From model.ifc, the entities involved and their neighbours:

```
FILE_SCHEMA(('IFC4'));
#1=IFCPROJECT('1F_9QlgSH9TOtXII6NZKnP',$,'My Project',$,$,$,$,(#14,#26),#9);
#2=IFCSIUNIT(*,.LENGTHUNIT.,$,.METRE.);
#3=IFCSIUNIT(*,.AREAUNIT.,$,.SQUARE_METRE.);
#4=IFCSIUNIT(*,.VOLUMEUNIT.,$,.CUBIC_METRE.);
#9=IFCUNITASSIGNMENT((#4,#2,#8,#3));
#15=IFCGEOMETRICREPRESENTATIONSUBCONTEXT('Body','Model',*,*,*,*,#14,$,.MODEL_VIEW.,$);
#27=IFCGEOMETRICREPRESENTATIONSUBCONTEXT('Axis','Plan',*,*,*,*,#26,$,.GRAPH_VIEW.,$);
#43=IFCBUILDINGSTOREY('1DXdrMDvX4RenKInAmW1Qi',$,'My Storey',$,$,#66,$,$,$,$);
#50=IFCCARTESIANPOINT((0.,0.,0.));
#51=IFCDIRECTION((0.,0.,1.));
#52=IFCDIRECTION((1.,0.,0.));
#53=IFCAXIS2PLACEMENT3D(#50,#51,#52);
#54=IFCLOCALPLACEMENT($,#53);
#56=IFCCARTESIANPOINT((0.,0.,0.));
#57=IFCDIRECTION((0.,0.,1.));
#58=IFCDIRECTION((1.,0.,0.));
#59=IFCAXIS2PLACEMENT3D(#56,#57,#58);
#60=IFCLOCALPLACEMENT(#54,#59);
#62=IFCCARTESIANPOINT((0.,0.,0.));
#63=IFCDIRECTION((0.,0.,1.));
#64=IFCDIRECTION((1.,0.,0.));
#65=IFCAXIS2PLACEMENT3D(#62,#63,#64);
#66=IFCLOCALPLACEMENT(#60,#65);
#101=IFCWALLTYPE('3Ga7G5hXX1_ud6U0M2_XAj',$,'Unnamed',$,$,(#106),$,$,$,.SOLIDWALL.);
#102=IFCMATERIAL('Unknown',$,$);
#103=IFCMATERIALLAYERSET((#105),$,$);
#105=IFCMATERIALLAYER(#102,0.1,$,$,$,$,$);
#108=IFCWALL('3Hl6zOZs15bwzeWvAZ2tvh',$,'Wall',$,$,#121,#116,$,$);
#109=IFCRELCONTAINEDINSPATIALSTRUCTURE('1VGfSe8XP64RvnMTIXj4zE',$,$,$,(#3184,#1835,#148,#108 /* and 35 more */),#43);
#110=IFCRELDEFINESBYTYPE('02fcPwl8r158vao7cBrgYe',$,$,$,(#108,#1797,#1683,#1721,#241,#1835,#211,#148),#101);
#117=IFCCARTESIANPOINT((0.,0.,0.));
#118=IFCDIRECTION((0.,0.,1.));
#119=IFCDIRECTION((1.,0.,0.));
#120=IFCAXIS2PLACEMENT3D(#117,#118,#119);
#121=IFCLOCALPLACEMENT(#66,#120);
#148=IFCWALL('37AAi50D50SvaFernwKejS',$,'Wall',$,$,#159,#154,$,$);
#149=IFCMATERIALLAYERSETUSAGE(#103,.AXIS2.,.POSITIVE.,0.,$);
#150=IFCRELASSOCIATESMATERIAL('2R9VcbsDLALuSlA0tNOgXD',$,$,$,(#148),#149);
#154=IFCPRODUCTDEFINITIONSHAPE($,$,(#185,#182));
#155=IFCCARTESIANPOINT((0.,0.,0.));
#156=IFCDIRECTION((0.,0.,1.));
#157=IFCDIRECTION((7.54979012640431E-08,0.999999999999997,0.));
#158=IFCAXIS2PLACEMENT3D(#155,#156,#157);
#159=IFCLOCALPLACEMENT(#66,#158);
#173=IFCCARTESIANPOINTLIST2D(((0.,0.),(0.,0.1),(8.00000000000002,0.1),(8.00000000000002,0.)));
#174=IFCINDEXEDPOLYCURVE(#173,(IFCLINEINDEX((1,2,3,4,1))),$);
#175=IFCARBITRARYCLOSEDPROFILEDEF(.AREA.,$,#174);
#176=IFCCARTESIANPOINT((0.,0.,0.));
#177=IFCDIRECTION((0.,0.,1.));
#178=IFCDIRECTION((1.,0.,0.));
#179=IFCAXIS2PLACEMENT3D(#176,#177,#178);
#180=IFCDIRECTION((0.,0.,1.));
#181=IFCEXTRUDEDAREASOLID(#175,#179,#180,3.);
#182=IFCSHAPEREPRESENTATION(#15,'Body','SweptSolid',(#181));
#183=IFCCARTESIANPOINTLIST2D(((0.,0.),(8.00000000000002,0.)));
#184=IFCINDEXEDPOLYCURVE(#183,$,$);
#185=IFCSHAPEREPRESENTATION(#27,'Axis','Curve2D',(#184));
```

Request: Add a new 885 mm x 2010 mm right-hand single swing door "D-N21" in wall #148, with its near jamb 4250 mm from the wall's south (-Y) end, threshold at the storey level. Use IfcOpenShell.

```python
import numpy as np
import ifcopenshell
import ifcopenshell.api.feature
import ifcopenshell.api.geometry
import ifcopenshell.api.root
import ifcopenshell.api.spatial
import ifcopenshell.geom
import ifcopenshell.util.element
import ifcopenshell.util.placement
import ifcopenshell.util.representation
import ifcopenshell.util.shape
import ifcopenshell.util.unit

model = ifcopenshell.open("model.ifc")
unit_scale = ifcopenshell.util.unit.calculate_unit_scale(model)
settings = ifcopenshell.geom.settings()


def volume(element):
    """Net volume in cubic metres, openings subtracted."""
    shape = ifcopenshell.geom.create_shape(settings, element)
    return ifcopenshell.util.shape.get_volume(shape.geometry)


wall = model.by_guid("37AAi50D50SvaFernwKejS")
storey = ifcopenshell.util.element.get_container(wall, ifc_class="IfcBuildingStorey")
context = ifcopenshell.util.representation.get_context(model, "Model", "Body", "MODEL_VIEW")
before = volume(wall)

width, height, from_end, sill = 0.885, 2.01, 4.25, 0.0  # metres

# The wall runs along its own X axis, and the end named is its -X end.
wall_shape = ifcopenshell.geom.create_shape(settings, wall)
x, y, z = ifcopenshell.util.shape.get_vertices(wall_shape.geometry).T
start = x.min() + from_end
face, thickness = float(y.min()), float(y.max() - y.min())
wall_matrix = ifcopenshell.util.placement.get_local_placement(wall.ObjectPlacement)
level = ifcopenshell.util.placement.get_local_placement(storey.ObjectPlacement)[2, 3]


def in_wall(x, y):
    """Placement at x, y metres in the wall's axes, at sill height."""
    matrix = wall_matrix.copy()
    matrix[:, 3] = wall_matrix @ np.array([x / unit_scale, y / unit_scale, 0.0, 1.0])
    matrix[2, 3] = level + sill / unit_scale
    return matrix


# Opening: a box that overshoots both wall faces by 50 mm.
opening = ifcopenshell.api.root.create_entity(model, ifc_class="IfcOpeningElement", predefined_type="OPENING")
box = ifcopenshell.api.geometry.add_wall_representation(
    model, context=context, length=width, height=height, thickness=thickness + 0.1
)
ifcopenshell.api.geometry.assign_representation(model, product=opening, representation=box)
ifcopenshell.api.geometry.edit_object_placement(model, product=opening, matrix=in_wall(start, face - 0.05), is_si=False)
ifcopenshell.api.feature.add_feature(model, feature=opening, element=wall)

door = ifcopenshell.api.root.create_entity(model, ifc_class="IfcDoor", name="D-N21", predefined_type="DOOR")
door.OverallWidth, door.OverallHeight = width / unit_scale, height / unit_scale
door.OperationType = "SINGLE_SWING_RIGHT"
body = ifcopenshell.api.geometry.add_door_representation(
    model,
    context=context,
    overall_width=door.OverallWidth,
    overall_height=door.OverallHeight,
    operation_type="SINGLE_SWING_RIGHT",
    lining_properties={"LiningDepth": thickness / unit_scale, "ThresholdDepth": thickness / unit_scale},
)
ifcopenshell.api.geometry.assign_representation(model, product=door, representation=body)
ifcopenshell.api.spatial.assign_container(model, products=[door], relating_structure=storey)
ifcopenshell.api.feature.add_filling(model, opening=opening, element=door)

# The lining spans the wall, so the door starts at the wall face.
ifcopenshell.api.geometry.edit_object_placement(model, product=door, matrix=in_wall(start, face), is_si=False)

after = volume(wall)

print(f"wall volume {before:.3f} -> {after:.3f} m3")

model.write("model-out.ifc")
```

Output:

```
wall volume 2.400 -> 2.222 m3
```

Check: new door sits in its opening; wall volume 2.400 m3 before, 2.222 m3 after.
